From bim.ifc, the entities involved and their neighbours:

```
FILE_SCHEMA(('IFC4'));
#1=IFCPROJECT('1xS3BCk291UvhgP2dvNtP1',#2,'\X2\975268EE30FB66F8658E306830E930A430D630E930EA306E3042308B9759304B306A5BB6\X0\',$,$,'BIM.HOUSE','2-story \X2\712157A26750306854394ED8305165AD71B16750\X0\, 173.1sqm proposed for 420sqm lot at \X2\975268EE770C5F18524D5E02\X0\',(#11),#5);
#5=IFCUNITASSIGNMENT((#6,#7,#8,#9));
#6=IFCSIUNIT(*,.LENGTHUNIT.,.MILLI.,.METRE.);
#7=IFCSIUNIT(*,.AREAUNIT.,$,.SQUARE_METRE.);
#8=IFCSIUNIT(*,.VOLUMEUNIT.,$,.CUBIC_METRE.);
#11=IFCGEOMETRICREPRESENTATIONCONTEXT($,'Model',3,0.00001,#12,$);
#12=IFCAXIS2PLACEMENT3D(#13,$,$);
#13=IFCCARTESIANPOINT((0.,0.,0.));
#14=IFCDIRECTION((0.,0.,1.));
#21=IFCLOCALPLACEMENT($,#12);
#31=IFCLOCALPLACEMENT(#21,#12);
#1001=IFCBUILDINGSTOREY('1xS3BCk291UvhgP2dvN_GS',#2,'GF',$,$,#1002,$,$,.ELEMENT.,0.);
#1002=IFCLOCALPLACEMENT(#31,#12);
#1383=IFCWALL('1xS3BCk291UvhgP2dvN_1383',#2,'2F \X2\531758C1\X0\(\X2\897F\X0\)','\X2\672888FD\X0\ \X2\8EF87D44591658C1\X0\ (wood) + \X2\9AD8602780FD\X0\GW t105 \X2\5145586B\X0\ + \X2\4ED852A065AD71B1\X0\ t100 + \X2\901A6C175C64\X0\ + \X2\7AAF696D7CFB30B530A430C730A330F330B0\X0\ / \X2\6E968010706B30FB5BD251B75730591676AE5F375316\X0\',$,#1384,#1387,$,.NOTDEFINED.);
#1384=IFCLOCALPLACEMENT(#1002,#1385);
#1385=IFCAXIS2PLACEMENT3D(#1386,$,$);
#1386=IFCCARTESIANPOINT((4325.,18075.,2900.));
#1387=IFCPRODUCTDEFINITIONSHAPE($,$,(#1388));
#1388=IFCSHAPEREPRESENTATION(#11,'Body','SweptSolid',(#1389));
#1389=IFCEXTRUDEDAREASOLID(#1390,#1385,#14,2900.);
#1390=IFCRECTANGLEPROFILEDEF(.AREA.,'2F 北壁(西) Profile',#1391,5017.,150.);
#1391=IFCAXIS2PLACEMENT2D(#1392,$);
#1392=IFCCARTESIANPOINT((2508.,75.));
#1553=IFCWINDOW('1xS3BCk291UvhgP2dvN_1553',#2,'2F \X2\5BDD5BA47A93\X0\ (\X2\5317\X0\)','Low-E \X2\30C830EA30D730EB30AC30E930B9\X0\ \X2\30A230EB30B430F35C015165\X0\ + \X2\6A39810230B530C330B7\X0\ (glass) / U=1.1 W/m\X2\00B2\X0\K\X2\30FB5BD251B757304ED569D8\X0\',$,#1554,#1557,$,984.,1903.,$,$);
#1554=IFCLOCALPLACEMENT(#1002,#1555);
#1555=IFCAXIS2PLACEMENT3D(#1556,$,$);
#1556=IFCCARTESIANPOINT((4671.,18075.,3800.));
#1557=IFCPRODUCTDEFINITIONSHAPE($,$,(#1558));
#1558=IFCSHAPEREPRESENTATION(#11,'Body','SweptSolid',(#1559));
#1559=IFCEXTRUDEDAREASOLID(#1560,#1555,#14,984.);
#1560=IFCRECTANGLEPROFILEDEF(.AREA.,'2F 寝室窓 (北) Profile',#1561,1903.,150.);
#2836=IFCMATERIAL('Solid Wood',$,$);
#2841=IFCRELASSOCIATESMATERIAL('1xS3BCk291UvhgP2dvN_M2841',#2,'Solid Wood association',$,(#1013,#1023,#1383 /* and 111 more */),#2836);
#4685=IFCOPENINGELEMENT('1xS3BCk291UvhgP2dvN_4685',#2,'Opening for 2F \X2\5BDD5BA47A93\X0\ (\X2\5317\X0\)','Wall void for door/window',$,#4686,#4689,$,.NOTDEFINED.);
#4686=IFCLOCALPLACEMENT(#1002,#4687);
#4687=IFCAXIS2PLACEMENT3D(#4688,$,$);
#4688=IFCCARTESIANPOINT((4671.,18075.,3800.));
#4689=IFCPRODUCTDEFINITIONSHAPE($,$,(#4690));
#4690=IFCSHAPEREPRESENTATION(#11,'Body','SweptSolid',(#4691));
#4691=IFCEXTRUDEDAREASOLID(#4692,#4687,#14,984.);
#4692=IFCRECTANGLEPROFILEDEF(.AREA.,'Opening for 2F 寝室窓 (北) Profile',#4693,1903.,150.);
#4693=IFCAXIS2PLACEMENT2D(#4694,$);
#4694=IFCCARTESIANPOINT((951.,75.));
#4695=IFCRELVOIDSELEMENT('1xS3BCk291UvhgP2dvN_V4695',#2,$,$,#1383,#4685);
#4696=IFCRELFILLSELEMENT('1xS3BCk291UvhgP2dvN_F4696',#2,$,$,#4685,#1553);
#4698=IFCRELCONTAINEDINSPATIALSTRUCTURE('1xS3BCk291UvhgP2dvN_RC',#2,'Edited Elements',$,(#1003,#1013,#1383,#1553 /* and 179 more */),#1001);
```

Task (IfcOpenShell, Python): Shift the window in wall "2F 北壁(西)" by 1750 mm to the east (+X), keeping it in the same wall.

```python
import ifcopenshell
import ifcopenshell.api.geometry
import ifcopenshell.util.placement

model = ifcopenshell.open("bim.ifc")

window = model.by_guid("1xS3BCk291UvhgP2dvN_1553")
opening = window.FillsVoids[0].RelatingOpeningElement
wall = opening.VoidsElements[0].RelatingBuildingElement

wall_matrix = ifcopenshell.util.placement.get_local_placement(wall.ObjectPlacement)
shift = wall_matrix[:3, 0] * 1750.0
before = ifcopenshell.util.placement.get_local_placement(window.ObjectPlacement)[:3, 3].copy()

# The window is not placed relative to its opening, so move both.
for product in (opening, window):
    matrix = ifcopenshell.util.placement.get_local_placement(product.ObjectPlacement)
    matrix[:3, 3] += shift
    ifcopenshell.api.geometry.edit_object_placement(model, product=product, matrix=matrix, is_si=False)

after = ifcopenshell.util.placement.get_local_placement(window.ObjectPlacement)[:3, 3]
print("window moved by", (after - before).round(3) + 0.0)

model.write("bim_v2.ifc")
```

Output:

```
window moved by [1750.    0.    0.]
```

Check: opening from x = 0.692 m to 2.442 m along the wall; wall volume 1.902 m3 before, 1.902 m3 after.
